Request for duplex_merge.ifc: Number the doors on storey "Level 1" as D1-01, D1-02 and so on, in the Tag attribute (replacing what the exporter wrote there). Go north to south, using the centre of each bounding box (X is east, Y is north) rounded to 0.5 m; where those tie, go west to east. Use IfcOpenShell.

First a look at what the model holds.

```python
import ifcopenshell
import ifcopenshell.util.element
import ifcopenshell.util.placement

model = ifcopenshell.open("duplex_merge.ifc")
print(model.schema)
storey = next(s for s in model.by_type("IfcBuildingStorey") if s.Name == "Level 1")
doors = [e for e in ifcopenshell.util.element.get_decomposition(storey) if e.is_a("IfcDoor")]
for e in sorted(doors, key=lambda e: e.id()):
    origin = ifcopenshell.util.placement.get_local_placement(e.ObjectPlacement)[:3, 3]
    print(e.id(), e.Tag, e.Name, origin.round(2) + 0.0, sep=" | ")
```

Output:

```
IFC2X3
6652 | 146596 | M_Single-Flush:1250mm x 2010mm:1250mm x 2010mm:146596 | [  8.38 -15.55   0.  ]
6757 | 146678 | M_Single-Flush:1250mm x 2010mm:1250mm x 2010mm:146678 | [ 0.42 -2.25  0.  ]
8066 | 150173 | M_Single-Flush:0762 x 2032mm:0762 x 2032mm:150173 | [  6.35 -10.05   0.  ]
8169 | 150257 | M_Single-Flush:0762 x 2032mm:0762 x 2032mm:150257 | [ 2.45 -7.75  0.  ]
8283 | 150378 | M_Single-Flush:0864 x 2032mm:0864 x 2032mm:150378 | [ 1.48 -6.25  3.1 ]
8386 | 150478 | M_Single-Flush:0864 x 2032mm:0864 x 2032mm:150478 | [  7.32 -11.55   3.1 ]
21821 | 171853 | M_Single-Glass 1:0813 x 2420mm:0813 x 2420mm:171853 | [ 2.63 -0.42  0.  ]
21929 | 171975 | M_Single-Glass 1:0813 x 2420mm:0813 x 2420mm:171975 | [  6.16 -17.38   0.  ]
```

```python
import ifcopenshell
import ifcopenshell.geom
import ifcopenshell.util.element
import ifcopenshell.util.shape

model = ifcopenshell.open("duplex_merge.ifc")
settings = ifcopenshell.geom.settings()
settings.set("use-world-coords", True)


def centre(element):
    shape = ifcopenshell.geom.create_shape(settings, element)
    return ifcopenshell.util.shape.get_bbox_centroid(shape.geometry)


storey = next(s for s in model.by_type("IfcBuildingStorey") if s.Name == "Level 1")
doors = [e for e in ifcopenshell.util.element.get_decomposition(storey) if e.is_a("IfcDoor")]

# Insertion points can sit at a corner or the storey origin, so sort by the geometry (in metres).
centres = {e: centre(e) for e in doors}
doors.sort(key=lambda e: (-round(centres[e][1] / 0.5), centres[e][0]))

for i, e in enumerate(doors, start=1):
    number = f"D1-{i:02d}"
    e.Tag = number
    print(e.id(), number)

model.write("duplex_merge_rev.ifc")
```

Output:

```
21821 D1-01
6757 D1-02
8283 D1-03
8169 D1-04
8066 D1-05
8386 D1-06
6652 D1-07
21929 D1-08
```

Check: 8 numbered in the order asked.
